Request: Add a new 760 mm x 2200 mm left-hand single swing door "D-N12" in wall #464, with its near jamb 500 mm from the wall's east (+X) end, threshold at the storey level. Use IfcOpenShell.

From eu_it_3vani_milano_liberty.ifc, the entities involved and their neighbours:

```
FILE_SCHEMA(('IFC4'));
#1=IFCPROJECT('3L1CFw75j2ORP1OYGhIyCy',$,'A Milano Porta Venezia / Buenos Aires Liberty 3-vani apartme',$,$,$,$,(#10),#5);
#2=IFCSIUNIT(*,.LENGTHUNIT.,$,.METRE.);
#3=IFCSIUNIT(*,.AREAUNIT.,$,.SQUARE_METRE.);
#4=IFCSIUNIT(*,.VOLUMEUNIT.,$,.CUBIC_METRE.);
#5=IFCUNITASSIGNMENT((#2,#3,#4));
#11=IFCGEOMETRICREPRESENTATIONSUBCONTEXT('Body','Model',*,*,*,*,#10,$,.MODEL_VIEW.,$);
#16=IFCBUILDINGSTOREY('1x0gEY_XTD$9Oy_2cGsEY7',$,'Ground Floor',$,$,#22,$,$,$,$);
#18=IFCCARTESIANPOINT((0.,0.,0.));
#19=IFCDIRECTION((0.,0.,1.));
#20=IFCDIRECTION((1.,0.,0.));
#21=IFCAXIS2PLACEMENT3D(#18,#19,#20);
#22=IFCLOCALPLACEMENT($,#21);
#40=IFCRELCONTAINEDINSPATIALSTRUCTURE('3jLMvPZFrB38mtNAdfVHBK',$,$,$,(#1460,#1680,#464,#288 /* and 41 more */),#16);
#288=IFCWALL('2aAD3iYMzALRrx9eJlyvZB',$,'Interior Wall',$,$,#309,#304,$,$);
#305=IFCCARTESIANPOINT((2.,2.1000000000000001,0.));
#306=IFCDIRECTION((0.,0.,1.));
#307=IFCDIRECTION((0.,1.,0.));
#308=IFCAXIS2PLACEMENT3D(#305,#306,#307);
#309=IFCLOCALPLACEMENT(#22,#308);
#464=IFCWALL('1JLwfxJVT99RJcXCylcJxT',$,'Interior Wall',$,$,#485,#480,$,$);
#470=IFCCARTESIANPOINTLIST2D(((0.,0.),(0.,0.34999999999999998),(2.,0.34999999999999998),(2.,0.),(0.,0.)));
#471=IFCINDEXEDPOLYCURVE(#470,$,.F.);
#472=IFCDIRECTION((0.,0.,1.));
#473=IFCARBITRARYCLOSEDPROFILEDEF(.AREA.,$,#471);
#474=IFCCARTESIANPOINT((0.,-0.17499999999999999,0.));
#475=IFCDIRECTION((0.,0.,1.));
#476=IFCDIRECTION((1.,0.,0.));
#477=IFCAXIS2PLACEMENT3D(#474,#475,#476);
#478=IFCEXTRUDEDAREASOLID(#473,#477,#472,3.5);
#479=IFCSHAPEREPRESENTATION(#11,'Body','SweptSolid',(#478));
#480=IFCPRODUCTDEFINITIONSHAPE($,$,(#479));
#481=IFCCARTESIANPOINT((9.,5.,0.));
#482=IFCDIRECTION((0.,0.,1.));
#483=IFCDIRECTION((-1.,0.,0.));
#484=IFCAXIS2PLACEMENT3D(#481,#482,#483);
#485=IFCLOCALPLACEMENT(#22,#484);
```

```python
import numpy as np
import ifcopenshell
import ifcopenshell.api.feature
import ifcopenshell.api.geometry
import ifcopenshell.api.root
import ifcopenshell.api.spatial
import ifcopenshell.geom
import ifcopenshell.util.element
import ifcopenshell.util.placement
import ifcopenshell.util.representation
import ifcopenshell.util.shape
import ifcopenshell.util.unit

model = ifcopenshell.open("eu_it_3vani_milano_liberty.ifc")
unit_scale = ifcopenshell.util.unit.calculate_unit_scale(model)
settings = ifcopenshell.geom.settings()


def volume(element):
    """Net volume in cubic metres, openings subtracted."""
    shape = ifcopenshell.geom.create_shape(settings, element)
    return ifcopenshell.util.shape.get_volume(shape.geometry)


wall = model.by_guid("1JLwfxJVT99RJcXCylcJxT")
storey = ifcopenshell.util.element.get_container(wall, ifc_class="IfcBuildingStorey")
context = ifcopenshell.util.representation.get_context(model, "Model", "Body", "MODEL_VIEW")
before = volume(wall)

width, height, from_end, sill = 0.76, 2.2, 0.5, 0.0  # metres

# The wall runs along its own X axis, and the end named is its -X end.
wall_shape = ifcopenshell.geom.create_shape(settings, wall)
x, y, z = ifcopenshell.util.shape.get_vertices(wall_shape.geometry).T
start = x.min() + from_end
face, thickness = float(y.min()), float(y.max() - y.min())
wall_matrix = ifcopenshell.util.placement.get_local_placement(wall.ObjectPlacement)
level = ifcopenshell.util.placement.get_local_placement(storey.ObjectPlacement)[2, 3]


def in_wall(x, y):
    """Placement at x, y metres in the wall's axes, at sill height."""
    matrix = wall_matrix.copy()
    matrix[:, 3] = wall_matrix @ np.array([x / unit_scale, y / unit_scale, 0.0, 1.0])
    matrix[2, 3] = level + sill / unit_scale
    return matrix


# Opening: a box that overshoots both wall faces by 50 mm.
opening = ifcopenshell.api.root.create_entity(model, ifc_class="IfcOpeningElement", predefined_type="OPENING")
box = ifcopenshell.api.geometry.add_wall_representation(
    model, context=context, length=width, height=height, thickness=thickness + 0.1
)
ifcopenshell.api.geometry.assign_representation(model, product=opening, representation=box)
ifcopenshell.api.geometry.edit_object_placement(model, product=opening, matrix=in_wall(start, face - 0.05), is_si=False)
ifcopenshell.api.feature.add_feature(model, feature=opening, element=wall)

door = ifcopenshell.api.root.create_entity(model, ifc_class="IfcDoor", name="D-N12", predefined_type="DOOR")
door.OverallWidth, door.OverallHeight = width / unit_scale, height / unit_scale
door.OperationType = "SINGLE_SWING_LEFT"
body = ifcopenshell.api.geometry.add_door_representation(
    model,
    context=context,
    overall_width=door.OverallWidth,
    overall_height=door.OverallHeight,
    operation_type="SINGLE_SWING_LEFT",
    lining_properties={"LiningDepth": thickness / unit_scale, "ThresholdDepth": thickness / unit_scale},
)
ifcopenshell.api.geometry.assign_representation(model, product=door, representation=body)
ifcopenshell.api.spatial.assign_container(model, products=[door], relating_structure=storey)
ifcopenshell.api.feature.add_filling(model, opening=opening, element=door)

# The lining spans the wall, so the door starts at the wall face.
ifcopenshell.api.geometry.edit_object_placement(model, product=door, matrix=in_wall(start, face), is_si=False)

after = volume(wall)

print(f"wall volume {before:.3f} -> {after:.3f} m3")

model.write("eu_it_3vani_milano_liberty-out.ifc")
```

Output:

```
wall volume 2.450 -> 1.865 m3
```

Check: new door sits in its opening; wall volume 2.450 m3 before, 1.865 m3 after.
